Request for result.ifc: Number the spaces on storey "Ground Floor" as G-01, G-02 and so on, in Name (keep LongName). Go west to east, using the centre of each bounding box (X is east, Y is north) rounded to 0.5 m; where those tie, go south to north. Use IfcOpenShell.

First a look at what the model holds.

```python
import ifcopenshell
import ifcopenshell.util.element
import ifcopenshell.util.placement

model = ifcopenshell.open("result.ifc")
print(model.schema)
storey = next(s for s in model.by_type("IfcBuildingStorey") if s.Name == "Ground Floor")
spaces = [e for e in ifcopenshell.util.element.get_decomposition(storey) if e.is_a("IfcSpace")]
for e in sorted(spaces, key=lambda e: e.id()):
    origin = ifcopenshell.util.placement.get_local_placement(e.ObjectPlacement)[:3, 3]
    print(e.id(), e.Name, e.LongName, origin.round(2) + 0.0, sep=" | ")
```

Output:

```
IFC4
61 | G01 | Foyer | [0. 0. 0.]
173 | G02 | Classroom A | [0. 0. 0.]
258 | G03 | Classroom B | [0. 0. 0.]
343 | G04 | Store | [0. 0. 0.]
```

```python
import ifcopenshell
import ifcopenshell.geom
import ifcopenshell.util.element
import ifcopenshell.util.shape

model = ifcopenshell.open("result.ifc")
settings = ifcopenshell.geom.settings()
settings.set("use-world-coords", True)


def centre(element):
    shape = ifcopenshell.geom.create_shape(settings, element)
    return ifcopenshell.util.shape.get_bbox_centroid(shape.geometry)


storey = next(s for s in model.by_type("IfcBuildingStorey") if s.Name == "Ground Floor")
spaces = [e for e in ifcopenshell.util.element.get_decomposition(storey) if e.is_a("IfcSpace")]

# Insertion points can sit at a corner or the storey origin, so sort by the geometry (in metres).
centres = {e: centre(e) for e in spaces}
spaces.sort(key=lambda e: (round(centres[e][0] / 0.5), centres[e][1]))

for i, e in enumerate(spaces, start=1):
    number = f"G-{i:02d}"
    e.Name = number
    print(e.id(), number)

model.write("result-out.ifc")
```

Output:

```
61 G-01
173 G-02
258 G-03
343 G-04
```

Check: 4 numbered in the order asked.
